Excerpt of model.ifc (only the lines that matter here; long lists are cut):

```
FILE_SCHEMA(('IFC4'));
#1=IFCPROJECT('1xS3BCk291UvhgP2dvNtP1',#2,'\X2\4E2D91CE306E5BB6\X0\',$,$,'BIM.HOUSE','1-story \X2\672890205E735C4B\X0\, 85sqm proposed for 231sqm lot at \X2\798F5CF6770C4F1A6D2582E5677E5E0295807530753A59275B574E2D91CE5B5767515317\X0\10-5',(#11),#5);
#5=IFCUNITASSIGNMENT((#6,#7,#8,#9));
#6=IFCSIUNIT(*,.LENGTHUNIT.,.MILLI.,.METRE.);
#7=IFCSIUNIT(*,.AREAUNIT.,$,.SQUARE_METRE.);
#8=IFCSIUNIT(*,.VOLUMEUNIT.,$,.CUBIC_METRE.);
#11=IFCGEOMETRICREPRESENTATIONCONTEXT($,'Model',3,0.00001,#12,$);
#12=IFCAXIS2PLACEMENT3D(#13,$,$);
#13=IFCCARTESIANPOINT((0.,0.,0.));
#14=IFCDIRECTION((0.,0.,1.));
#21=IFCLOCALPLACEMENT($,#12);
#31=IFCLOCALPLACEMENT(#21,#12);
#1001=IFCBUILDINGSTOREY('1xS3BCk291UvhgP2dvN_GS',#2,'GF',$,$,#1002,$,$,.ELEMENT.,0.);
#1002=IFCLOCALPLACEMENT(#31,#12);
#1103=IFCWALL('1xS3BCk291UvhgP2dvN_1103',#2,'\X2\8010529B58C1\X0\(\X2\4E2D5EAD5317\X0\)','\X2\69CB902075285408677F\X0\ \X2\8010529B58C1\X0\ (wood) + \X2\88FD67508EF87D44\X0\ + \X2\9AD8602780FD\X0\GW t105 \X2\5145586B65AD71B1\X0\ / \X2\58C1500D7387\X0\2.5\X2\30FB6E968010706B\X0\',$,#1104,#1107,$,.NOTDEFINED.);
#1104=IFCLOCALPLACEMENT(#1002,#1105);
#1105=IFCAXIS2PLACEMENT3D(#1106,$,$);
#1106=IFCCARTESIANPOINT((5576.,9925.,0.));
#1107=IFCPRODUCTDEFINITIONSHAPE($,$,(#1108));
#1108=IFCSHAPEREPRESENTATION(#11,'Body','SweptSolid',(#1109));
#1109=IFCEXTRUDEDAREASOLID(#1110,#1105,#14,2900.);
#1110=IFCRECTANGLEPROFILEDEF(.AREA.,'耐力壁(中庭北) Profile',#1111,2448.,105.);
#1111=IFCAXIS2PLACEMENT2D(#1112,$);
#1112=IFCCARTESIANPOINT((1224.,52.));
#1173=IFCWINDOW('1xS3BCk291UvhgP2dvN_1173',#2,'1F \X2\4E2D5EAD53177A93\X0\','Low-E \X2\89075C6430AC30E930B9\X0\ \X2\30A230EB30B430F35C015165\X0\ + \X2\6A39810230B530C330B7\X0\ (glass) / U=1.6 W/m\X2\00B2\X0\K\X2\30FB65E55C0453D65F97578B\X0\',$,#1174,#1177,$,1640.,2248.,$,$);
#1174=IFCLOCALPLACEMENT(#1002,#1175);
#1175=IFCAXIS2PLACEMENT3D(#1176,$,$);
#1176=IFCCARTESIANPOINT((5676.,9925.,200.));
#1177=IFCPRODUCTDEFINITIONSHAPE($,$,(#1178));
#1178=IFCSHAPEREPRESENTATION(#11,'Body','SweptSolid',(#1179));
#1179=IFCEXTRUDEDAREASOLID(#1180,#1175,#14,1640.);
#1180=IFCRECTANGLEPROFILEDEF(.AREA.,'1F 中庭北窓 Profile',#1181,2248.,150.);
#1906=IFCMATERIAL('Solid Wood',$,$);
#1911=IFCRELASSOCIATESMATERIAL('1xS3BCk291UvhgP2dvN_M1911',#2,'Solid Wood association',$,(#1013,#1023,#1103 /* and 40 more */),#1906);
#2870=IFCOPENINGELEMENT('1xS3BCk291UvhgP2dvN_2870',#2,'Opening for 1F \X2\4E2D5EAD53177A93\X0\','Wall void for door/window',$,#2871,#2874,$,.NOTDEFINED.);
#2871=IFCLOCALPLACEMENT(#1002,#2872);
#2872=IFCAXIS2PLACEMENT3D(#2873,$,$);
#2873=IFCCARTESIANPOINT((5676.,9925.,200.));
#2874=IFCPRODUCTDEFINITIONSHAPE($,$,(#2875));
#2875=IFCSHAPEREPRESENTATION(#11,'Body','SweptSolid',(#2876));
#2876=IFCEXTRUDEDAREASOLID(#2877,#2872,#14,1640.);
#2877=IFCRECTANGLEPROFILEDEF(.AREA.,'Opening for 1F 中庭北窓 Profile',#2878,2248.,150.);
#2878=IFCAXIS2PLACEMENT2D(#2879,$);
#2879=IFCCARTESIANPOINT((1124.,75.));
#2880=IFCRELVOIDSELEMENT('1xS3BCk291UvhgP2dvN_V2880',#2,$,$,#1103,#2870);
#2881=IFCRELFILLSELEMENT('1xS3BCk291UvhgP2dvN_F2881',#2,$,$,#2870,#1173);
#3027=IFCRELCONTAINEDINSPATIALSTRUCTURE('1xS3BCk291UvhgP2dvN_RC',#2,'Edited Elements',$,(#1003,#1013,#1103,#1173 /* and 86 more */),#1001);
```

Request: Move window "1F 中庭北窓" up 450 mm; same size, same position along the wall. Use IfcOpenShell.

```python
import numpy as np
import ifcopenshell
import ifcopenshell.api.geometry
import ifcopenshell.util.placement
import ifcopenshell.util.unit

model = ifcopenshell.open("model.ifc")
unit_scale = ifcopenshell.util.unit.calculate_unit_scale(model)

window = model.by_guid("1xS3BCk291UvhgP2dvN_1173")
opening = window.FillsVoids[0].RelatingOpeningElement
dz = 450.0

shift = np.array([0.0, 0.0, dz])
# The window is not placed relative to its opening, so move both.
for product in (opening, window):
    matrix = ifcopenshell.util.placement.get_local_placement(product.ObjectPlacement)
    matrix[:3, 3] += shift
    ifcopenshell.api.geometry.edit_object_placement(model, product=product, matrix=matrix, is_si=False)

print(f"moved by {dz * unit_scale:+.3f} m")

model.write("model_v2.ifc")
```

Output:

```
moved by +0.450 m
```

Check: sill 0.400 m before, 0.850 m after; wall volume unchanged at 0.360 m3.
